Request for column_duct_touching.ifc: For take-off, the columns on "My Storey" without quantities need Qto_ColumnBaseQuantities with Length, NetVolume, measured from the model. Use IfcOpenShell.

First a look at what the model holds.

```python
import ifcopenshell
import ifcopenshell.util.element
import ifcopenshell.util.unit

model = ifcopenshell.open("column_duct_touching.ifc")
print(model.schema)
for unit_type in ("LENGTHUNIT", "AREAUNIT", "VOLUMEUNIT"):
    print(unit_type, ifcopenshell.util.unit.calculate_unit_scale(model, unit_type))
storey = next(s for s in model.by_type("IfcBuildingStorey") if s.Name == "My Storey")
columns = [e for e in ifcopenshell.util.element.get_decomposition(storey) if e.is_a("IfcColumn")]
for e in sorted(columns, key=lambda e: e.id()):
    print(e.id(), e.is_a(), e.Name, list(ifcopenshell.util.element.get_psets(e, qtos_only=True)), sep=" | ")
```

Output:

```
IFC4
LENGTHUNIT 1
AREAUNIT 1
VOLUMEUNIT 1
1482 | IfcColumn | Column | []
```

```python
import ifcopenshell
import ifcopenshell.api.pset
import ifcopenshell.geom
import ifcopenshell.util.element
import ifcopenshell.util.shape
import ifcopenshell.util.unit

model = ifcopenshell.open("column_duct_touching.ifc")
unit_scale = ifcopenshell.util.unit.calculate_unit_scale(model)
volume_scale = ifcopenshell.util.unit.calculate_unit_scale(model, "VOLUMEUNIT")
settings = ifcopenshell.geom.settings()

storey = next(s for s in model.by_type("IfcBuildingStorey") if s.Name == "My Storey")
columns = [e for e in ifcopenshell.util.element.get_decomposition(storey) if e.is_a("IfcColumn")]

for e in sorted(columns, key=lambda e: e.id()):
    if ifcopenshell.util.element.get_psets(e, qtos_only=True, should_inherit=False):
        continue
    # Geometry comes back in metres, in the element's own axes.
    shape = ifcopenshell.geom.create_shape(settings, e)
    values = {
        "Length": ifcopenshell.util.shape.get_z(shape.geometry) / unit_scale,
        "NetVolume": ifcopenshell.util.shape.get_volume(shape.geometry) / volume_scale,
    }
    qto = ifcopenshell.api.pset.add_qto(model, product=e, name="Qto_ColumnBaseQuantities")
    ifcopenshell.api.pset.edit_qto(model, qto=qto, properties=values)
    print(e.id(), {k: round(v, 3) for k, v in values.items()})

model.write("column_duct_touching_rev.ifc")
```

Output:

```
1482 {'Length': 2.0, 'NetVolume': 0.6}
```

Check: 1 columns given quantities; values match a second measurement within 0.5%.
